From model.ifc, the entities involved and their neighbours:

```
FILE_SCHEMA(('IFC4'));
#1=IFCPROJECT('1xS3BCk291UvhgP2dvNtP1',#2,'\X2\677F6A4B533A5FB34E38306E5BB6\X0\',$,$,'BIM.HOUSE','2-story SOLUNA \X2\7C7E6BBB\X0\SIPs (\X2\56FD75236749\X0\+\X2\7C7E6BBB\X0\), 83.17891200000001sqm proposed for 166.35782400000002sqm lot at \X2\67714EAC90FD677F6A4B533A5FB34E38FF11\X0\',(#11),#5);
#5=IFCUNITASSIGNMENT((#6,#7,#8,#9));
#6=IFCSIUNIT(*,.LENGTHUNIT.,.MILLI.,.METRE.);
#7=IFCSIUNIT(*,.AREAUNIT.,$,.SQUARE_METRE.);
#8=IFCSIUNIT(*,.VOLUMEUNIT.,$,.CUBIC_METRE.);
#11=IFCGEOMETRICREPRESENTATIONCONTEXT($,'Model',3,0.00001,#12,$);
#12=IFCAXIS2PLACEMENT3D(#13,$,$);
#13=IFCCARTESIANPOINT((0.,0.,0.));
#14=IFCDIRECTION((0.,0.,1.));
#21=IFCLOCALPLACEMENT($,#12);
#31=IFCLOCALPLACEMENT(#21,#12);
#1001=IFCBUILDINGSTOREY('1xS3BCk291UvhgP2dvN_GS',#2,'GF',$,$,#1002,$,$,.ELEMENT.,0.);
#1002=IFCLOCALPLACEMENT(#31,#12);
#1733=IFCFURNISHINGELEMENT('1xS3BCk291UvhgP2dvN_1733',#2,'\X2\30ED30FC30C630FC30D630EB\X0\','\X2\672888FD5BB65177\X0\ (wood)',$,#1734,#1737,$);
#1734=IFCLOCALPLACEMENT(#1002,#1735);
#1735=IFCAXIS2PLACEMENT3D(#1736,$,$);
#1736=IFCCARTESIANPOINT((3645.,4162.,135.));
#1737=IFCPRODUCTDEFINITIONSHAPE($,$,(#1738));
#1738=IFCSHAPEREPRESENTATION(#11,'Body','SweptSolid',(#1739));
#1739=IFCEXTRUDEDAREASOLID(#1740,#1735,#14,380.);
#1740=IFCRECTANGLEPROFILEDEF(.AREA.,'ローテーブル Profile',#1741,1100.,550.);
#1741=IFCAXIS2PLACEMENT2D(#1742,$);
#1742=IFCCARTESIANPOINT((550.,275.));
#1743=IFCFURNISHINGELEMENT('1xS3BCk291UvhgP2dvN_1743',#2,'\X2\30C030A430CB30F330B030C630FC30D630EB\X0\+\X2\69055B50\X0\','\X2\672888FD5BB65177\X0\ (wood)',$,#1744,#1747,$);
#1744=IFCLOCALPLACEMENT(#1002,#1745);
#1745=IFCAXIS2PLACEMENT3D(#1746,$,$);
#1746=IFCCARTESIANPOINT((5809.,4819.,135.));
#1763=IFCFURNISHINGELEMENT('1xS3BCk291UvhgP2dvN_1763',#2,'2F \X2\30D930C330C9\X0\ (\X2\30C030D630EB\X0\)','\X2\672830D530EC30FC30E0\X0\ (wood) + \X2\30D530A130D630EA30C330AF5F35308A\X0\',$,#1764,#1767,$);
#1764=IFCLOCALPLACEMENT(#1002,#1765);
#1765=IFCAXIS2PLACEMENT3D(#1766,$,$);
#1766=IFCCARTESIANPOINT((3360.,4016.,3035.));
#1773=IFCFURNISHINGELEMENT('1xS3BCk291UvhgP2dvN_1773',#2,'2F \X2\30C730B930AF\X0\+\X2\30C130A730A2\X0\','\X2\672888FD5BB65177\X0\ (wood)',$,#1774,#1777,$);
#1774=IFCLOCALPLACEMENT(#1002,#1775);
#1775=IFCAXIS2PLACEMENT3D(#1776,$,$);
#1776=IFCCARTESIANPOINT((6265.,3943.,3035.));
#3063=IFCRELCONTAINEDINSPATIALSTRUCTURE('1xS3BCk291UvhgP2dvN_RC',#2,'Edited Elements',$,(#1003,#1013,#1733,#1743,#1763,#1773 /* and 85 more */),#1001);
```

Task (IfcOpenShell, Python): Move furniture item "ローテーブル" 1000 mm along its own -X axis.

```python
import ifcopenshell
import ifcopenshell.api.geometry
import ifcopenshell.util.placement

model = ifcopenshell.open("model.ifc")

item = model.by_guid("1xS3BCk291UvhgP2dvN_1733")
matrix = ifcopenshell.util.placement.get_local_placement(item.ObjectPlacement)
matrix[:3, 3] -= matrix[:3, 0] * 1000.0
ifcopenshell.api.geometry.edit_object_placement(model, product=item, matrix=matrix, is_si=False)

print(ifcopenshell.util.placement.get_local_placement(item.ObjectPlacement).round(3) + 0.0)

model.write("model_rev.ifc")
```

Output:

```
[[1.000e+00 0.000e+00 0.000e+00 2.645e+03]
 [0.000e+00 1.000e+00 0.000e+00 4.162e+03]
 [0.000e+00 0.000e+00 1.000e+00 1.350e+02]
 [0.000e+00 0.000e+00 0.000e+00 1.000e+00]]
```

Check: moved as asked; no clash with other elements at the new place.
